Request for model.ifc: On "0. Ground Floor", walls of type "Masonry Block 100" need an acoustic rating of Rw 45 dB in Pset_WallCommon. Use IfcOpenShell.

First a look at what the model holds.

```python
import ifcopenshell
import ifcopenshell.util.element

model = ifcopenshell.open("model.ifc")
print(model.schema)
storey = next(s for s in model.by_type("IfcBuildingStorey") if s.Name == "0. Ground Floor")
walls = [e for e in ifcopenshell.util.element.get_decomposition(storey) if e.is_a("IfcWall")]
seen = {}
for e in walls:
    element_type = ifcopenshell.util.element.get_type(e)
    key = (element_type.Name if element_type != e and element_type else None, ifcopenshell.util.element.get_pset(e, "Pset_WallCommon", "AcousticRating"))
    seen[key] = seen.get(key, 0) + 1
for (name, value), count in sorted(seen.items(), key=str):
    print(count, "x", name, "|", value)
```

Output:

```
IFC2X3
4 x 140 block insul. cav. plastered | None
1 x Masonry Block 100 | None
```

```python
import ifcopenshell
import ifcopenshell.api.pset
import ifcopenshell.util.element

model = ifcopenshell.open("model.ifc")

storey = next(s for s in model.by_type("IfcBuildingStorey") if s.Name == "0. Ground Floor")
walls = [e for e in ifcopenshell.util.element.get_decomposition(storey) if e.is_a("IfcWall")]

count = 0
for e in walls:
    element_type = ifcopenshell.util.element.get_type(e)
    if element_type in (None, e) or element_type.Name != "Masonry Block 100":
        continue
    # add_pset returns the element's existing set when there is one.
    pset = ifcopenshell.api.pset.add_pset(model, product=e, name="Pset_WallCommon")
    ifcopenshell.api.pset.edit_pset(model, pset=pset, properties={"AcousticRating": "Rw 45 dB"})
    count += 1

print(count, "walls updated")

model.write("model_edited.ifc")
```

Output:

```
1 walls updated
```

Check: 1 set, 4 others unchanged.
